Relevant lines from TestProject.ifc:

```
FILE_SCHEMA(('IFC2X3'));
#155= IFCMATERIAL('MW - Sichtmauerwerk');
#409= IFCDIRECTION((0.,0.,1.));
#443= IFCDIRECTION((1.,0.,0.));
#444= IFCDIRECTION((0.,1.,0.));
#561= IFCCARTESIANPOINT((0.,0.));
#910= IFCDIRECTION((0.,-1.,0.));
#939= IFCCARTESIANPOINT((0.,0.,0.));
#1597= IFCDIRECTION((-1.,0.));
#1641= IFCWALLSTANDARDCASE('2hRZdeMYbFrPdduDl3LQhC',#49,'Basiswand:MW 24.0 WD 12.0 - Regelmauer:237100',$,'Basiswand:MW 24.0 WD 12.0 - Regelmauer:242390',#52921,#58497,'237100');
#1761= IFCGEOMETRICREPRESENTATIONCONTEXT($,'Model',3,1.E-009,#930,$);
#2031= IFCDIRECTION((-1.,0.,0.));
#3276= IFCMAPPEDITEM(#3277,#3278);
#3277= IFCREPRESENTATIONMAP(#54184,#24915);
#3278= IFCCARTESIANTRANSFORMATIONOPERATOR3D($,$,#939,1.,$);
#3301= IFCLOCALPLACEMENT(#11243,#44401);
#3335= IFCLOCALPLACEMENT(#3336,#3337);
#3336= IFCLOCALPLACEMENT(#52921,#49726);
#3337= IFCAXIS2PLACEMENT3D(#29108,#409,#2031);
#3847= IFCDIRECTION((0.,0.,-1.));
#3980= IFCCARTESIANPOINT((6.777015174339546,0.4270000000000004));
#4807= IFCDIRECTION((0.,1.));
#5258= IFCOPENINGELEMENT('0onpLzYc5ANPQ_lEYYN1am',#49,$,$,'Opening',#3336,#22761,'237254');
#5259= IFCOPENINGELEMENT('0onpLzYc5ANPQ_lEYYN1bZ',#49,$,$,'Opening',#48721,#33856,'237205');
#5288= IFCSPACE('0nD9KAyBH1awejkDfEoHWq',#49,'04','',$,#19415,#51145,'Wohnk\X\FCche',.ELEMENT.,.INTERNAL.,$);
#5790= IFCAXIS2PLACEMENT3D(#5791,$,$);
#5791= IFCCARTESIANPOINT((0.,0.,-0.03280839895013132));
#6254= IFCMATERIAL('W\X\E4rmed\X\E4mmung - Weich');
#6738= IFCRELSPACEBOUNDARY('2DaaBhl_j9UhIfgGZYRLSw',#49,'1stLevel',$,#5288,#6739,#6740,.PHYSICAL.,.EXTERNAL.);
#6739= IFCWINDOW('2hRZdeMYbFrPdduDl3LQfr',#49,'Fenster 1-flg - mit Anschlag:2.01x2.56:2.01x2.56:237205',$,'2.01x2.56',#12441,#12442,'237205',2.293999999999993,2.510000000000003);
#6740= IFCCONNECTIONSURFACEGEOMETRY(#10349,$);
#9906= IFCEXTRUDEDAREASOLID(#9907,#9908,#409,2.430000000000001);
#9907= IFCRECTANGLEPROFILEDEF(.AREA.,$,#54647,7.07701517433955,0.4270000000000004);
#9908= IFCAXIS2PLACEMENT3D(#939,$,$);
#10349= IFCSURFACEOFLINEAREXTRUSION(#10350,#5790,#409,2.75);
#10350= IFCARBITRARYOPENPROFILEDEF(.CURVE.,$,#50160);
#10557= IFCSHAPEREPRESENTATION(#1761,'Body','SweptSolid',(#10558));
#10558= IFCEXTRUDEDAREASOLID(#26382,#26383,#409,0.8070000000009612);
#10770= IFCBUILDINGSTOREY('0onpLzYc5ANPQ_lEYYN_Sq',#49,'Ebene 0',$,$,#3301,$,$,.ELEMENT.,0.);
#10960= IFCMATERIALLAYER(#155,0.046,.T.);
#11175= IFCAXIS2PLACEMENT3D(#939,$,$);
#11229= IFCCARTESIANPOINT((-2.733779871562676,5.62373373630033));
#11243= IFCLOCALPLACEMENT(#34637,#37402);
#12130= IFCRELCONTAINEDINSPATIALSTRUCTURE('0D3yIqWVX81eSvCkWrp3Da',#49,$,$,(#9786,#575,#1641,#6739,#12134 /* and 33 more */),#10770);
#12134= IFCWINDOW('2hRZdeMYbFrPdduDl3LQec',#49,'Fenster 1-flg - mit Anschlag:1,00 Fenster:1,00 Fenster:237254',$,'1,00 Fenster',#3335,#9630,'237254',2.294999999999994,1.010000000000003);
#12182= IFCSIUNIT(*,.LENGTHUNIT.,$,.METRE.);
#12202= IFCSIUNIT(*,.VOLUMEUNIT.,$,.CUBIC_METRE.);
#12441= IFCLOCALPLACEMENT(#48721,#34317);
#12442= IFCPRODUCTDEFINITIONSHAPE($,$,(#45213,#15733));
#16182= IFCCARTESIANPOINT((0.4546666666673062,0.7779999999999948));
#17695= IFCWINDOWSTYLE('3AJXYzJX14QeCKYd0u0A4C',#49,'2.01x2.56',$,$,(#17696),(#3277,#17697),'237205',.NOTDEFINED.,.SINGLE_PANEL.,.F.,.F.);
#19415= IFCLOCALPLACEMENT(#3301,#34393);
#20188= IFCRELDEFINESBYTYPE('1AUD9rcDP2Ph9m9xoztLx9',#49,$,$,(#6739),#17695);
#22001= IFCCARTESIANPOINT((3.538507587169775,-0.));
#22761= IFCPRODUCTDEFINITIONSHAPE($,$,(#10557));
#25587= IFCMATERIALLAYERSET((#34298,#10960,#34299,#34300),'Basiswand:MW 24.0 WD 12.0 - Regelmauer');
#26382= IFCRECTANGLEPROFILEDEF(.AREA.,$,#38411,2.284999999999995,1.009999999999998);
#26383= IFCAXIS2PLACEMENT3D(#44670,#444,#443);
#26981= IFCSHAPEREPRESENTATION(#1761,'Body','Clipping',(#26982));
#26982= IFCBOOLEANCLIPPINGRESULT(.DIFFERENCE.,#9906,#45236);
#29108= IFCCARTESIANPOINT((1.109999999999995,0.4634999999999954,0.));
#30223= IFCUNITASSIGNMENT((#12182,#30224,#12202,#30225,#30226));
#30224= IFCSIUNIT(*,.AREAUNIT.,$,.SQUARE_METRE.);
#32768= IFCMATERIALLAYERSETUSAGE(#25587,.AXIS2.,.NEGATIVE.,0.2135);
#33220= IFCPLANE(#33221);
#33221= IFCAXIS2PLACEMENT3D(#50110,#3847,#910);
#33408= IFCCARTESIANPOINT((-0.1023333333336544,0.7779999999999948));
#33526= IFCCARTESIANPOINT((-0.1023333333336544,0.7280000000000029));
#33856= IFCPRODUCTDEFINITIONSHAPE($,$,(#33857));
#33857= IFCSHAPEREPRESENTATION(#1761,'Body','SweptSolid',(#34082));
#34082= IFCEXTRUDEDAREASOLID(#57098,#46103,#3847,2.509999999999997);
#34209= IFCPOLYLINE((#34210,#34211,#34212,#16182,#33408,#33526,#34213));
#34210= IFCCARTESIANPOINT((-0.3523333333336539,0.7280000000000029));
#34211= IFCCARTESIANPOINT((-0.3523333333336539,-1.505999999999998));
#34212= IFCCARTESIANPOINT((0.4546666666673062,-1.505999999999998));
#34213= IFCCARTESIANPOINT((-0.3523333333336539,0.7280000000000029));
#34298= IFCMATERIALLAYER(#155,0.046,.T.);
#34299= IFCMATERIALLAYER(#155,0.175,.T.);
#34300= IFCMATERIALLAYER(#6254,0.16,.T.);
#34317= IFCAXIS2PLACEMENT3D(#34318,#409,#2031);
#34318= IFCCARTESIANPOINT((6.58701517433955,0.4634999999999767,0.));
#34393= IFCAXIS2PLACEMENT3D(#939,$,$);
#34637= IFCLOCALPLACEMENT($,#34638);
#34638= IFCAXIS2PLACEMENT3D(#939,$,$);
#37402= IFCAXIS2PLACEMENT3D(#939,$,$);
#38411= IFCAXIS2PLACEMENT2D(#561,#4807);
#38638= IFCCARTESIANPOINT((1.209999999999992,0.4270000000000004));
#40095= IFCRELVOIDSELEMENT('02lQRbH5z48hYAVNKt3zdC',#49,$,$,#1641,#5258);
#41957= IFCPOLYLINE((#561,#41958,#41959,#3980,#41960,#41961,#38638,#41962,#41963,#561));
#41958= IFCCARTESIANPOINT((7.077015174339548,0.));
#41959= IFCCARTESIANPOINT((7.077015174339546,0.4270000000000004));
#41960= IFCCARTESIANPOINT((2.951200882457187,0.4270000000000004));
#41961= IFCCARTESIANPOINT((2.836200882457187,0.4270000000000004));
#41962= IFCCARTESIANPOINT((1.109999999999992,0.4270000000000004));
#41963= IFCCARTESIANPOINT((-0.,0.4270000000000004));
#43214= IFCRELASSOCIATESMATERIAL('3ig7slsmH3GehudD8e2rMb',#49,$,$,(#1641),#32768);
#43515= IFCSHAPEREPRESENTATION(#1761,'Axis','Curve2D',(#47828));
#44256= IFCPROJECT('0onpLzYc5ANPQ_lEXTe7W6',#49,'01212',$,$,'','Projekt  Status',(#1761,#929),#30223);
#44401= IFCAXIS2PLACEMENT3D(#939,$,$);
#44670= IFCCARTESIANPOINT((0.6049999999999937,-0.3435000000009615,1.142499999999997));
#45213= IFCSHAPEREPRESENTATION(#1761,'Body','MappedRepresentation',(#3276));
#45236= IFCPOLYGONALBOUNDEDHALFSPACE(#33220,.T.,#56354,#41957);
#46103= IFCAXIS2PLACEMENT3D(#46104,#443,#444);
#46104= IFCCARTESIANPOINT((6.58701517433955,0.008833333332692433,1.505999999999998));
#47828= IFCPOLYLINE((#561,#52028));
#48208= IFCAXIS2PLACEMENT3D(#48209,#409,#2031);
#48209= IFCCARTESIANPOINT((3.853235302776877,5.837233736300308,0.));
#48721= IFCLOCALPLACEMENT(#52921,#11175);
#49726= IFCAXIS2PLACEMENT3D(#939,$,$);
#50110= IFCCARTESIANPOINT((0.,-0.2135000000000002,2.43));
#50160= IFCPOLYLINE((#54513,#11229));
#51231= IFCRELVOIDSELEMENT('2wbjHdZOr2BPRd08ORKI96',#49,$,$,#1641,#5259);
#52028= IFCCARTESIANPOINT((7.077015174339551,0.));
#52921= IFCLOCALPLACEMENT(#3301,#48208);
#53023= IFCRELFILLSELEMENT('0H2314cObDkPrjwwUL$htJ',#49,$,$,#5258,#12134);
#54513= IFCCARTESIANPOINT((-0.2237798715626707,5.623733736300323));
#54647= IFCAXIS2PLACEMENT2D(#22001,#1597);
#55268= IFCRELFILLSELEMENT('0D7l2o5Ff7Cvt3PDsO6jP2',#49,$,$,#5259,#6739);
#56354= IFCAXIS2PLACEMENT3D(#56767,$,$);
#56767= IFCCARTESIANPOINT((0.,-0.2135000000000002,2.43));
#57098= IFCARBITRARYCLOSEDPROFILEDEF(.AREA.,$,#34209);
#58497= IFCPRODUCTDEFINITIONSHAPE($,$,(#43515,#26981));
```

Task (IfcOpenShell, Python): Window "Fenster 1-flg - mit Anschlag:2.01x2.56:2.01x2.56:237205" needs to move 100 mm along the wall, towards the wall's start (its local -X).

```python
import numpy as np
import ifcopenshell
import ifcopenshell.api.geometry
import ifcopenshell.util.placement
import ifcopenshell.util.unit

model = ifcopenshell.open("TestProject.ifc")
unit_scale = ifcopenshell.util.unit.calculate_unit_scale(model)

window = model.by_id(6739)
opening = window.FillsVoids[0].RelatingOpeningElement
wall = opening.VoidsElements[0].RelatingBuildingElement

wall_matrix = ifcopenshell.util.placement.get_local_placement(wall.ObjectPlacement)
shift = wall_matrix[:3, 0] * -0.1 / unit_scale
before = ifcopenshell.util.placement.get_local_placement(window.ObjectPlacement)[:3, 3].copy()

# The window is placed relative to its opening, so it follows when the opening moves.
matrix = ifcopenshell.util.placement.get_local_placement(opening.ObjectPlacement)
matrix[:3, 3] += shift
ifcopenshell.api.geometry.edit_object_placement(
    model, product=opening, matrix=matrix, is_si=False, should_transform_children=True
)

# Space boundary surfaces are stored in each space's coordinates; move them too.
for rel in window.ProvidesBoundaries:
    if not rel.ConnectionGeometry:
        continue
    surface = rel.ConnectionGeometry.SurfaceOnRelatingElement
    space_matrix = ifcopenshell.util.placement.get_local_placement(rel.RelatingSpace.ObjectPlacement)
    point = np.array(surface.Position.Location.Coordinates) + space_matrix[:3, :3].T @ shift
    surface.Position = model.createIfcAxis2Placement3D(
        model.createIfcCartesianPoint(point.tolist()), surface.Position.Axis, surface.Position.RefDirection
    )

after = ifcopenshell.util.placement.get_local_placement(window.ObjectPlacement)[:3, 3]
print("window moved by", (after - before).round(3) + 0.0)

model.write("TestProject_rev.ifc")
```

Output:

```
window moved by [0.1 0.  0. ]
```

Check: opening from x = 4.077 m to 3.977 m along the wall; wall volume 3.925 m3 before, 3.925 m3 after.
